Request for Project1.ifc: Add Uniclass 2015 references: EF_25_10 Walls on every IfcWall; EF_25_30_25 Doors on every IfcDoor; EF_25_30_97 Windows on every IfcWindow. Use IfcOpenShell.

First a look at what the model holds.

```python
import ifcopenshell

model = ifcopenshell.open("Project1.ifc")
print(model.schema)
print("classifications:", [c.Name for c in model.by_type("IfcClassification")])
for ifc_class in ("IfcDoor", "IfcRoof", "IfcStair", "IfcWall", "IfcWindow"):
    print(ifc_class, len(model.by_type(ifc_class)))
```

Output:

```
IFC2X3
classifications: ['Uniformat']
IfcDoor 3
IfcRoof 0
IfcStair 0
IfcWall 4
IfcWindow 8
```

```python
import ifcopenshell
import ifcopenshell.api.classification

model = ifcopenshell.open("Project1.ifc")

# IFC2X3 requires Source and Edition and has no link from the project to the system.
system = model.create_entity("IfcClassification", Source="NBS", Edition="2015", Name="Uniclass 2015")

codes = {
    "IfcWall": ("EF_25_10", "Walls"),
    "IfcDoor": ("EF_25_30_25", "Doors"),
    "IfcWindow": ("EF_25_30_97", "Windows"),
}
for ifc_class, (code, name) in codes.items():
    products = model.by_type(ifc_class)
    ifcopenshell.api.classification.add_reference(
        model, products=products, classification=system, identification=code, name=name
    )
    print(code, len(products))

model.write("Project1_updated.ifc")
```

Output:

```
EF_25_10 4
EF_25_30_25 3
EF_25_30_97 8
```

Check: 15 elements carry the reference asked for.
